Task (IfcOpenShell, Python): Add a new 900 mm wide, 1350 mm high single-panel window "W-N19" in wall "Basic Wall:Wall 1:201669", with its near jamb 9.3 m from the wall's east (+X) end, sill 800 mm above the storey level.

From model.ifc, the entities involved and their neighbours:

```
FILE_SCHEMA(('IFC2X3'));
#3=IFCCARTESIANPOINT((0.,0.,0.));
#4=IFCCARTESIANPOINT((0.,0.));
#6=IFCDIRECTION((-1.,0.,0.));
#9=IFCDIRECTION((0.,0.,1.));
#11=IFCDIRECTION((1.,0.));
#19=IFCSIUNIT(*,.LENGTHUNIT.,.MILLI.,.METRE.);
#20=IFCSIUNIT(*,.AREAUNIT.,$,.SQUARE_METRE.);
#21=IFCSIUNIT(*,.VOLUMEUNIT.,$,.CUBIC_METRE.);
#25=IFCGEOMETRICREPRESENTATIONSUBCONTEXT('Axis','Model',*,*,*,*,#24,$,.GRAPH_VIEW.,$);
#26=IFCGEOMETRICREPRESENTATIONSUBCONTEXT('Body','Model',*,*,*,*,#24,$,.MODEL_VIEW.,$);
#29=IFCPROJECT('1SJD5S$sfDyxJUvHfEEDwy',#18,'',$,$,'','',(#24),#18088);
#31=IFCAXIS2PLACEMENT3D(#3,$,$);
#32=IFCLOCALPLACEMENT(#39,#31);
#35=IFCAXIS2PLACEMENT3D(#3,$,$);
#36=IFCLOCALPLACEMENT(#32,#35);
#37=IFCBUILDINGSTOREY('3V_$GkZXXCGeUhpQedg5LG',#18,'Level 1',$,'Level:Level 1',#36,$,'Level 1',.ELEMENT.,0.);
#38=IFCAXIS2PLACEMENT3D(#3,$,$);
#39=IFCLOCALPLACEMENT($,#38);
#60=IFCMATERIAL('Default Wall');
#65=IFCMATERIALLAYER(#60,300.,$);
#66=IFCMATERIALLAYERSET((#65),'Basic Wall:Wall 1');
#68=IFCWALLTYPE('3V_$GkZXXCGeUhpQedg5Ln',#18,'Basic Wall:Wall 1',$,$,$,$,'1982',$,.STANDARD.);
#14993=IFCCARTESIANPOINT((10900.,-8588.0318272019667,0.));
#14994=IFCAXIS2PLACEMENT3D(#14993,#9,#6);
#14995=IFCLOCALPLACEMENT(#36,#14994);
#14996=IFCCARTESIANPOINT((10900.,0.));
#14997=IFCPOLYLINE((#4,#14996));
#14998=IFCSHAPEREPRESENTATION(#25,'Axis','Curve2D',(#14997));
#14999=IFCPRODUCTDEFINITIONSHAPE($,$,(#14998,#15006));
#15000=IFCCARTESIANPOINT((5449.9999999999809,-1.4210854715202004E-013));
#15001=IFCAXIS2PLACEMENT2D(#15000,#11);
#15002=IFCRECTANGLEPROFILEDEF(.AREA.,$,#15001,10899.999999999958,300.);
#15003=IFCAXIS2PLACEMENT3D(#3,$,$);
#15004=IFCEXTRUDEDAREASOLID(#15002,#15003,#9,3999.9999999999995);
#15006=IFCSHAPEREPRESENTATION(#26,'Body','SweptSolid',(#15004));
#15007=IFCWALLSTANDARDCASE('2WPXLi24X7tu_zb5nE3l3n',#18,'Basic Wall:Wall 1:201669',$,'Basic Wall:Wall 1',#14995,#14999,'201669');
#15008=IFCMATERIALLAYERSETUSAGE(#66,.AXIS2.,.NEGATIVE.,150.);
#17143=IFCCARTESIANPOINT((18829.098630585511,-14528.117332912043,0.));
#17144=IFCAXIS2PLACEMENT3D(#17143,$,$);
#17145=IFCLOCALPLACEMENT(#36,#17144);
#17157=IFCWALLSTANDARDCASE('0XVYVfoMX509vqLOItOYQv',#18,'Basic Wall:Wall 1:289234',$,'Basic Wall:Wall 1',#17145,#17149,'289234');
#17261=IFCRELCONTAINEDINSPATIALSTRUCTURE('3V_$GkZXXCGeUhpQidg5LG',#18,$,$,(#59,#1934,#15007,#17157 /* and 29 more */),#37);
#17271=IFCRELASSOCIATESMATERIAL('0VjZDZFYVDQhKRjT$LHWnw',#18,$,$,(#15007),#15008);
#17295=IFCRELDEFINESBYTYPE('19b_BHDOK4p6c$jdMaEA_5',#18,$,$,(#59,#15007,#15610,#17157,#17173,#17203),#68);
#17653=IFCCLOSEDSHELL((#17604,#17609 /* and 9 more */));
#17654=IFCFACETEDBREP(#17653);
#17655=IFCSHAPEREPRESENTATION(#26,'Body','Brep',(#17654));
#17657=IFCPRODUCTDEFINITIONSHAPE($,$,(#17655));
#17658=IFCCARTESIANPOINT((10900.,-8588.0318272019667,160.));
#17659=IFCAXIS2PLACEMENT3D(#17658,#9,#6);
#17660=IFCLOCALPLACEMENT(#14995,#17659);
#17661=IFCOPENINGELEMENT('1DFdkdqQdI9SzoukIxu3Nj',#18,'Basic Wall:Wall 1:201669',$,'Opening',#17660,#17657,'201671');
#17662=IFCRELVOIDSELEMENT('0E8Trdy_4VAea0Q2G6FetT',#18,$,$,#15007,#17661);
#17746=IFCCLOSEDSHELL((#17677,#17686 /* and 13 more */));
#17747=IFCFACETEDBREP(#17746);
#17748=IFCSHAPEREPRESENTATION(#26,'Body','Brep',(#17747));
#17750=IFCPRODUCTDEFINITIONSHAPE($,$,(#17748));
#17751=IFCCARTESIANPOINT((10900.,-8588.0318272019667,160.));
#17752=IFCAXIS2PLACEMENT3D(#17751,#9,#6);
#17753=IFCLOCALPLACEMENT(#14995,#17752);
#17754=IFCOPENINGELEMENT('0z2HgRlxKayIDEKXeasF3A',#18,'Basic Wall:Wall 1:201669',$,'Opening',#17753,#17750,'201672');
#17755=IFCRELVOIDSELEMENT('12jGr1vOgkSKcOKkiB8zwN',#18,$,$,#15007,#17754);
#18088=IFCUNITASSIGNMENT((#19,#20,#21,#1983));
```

```python
import numpy as np
import ifcopenshell
import ifcopenshell.api.feature
import ifcopenshell.api.geometry
import ifcopenshell.api.root
import ifcopenshell.api.spatial
import ifcopenshell.api.type
import ifcopenshell.geom
import ifcopenshell.util.element
import ifcopenshell.util.placement
import ifcopenshell.util.representation
import ifcopenshell.util.shape
import ifcopenshell.util.unit

model = ifcopenshell.open("model.ifc")
unit_scale = ifcopenshell.util.unit.calculate_unit_scale(model)
settings = ifcopenshell.geom.settings()


def volume(element):
    """Net volume in cubic metres, openings subtracted."""
    shape = ifcopenshell.geom.create_shape(settings, element)
    return ifcopenshell.util.shape.get_volume(shape.geometry)


wall = model.by_guid("2WPXLi24X7tu_zb5nE3l3n")
storey = ifcopenshell.util.element.get_container(wall, ifc_class="IfcBuildingStorey")
context = ifcopenshell.util.representation.get_context(model, "Model", "Body", "MODEL_VIEW")
before = volume(wall)

width, height, from_end, sill = 0.9, 1.35, 9.3, 0.8  # metres

# The wall runs along its own X axis, and the end named is its -X end.
wall_shape = ifcopenshell.geom.create_shape(settings, wall)
x, y, z = ifcopenshell.util.shape.get_vertices(wall_shape.geometry).T
start = x.min() + from_end
face, thickness = float(y.min()), float(y.max() - y.min())
wall_matrix = ifcopenshell.util.placement.get_local_placement(wall.ObjectPlacement)
level = ifcopenshell.util.placement.get_local_placement(storey.ObjectPlacement)[2, 3]


def in_wall(x, y):
    """Placement at x, y metres in the wall's axes, at sill height."""
    matrix = wall_matrix.copy()
    matrix[:, 3] = wall_matrix @ np.array([x / unit_scale, y / unit_scale, 0.0, 1.0])
    matrix[2, 3] = level + sill / unit_scale
    return matrix


# Opening: a box that overshoots both wall faces by 50 mm.
opening = ifcopenshell.api.root.create_entity(model, ifc_class="IfcOpeningElement")
box = ifcopenshell.api.geometry.add_wall_representation(
    model, context=context, length=width, height=height, thickness=thickness + 0.1
)
ifcopenshell.api.geometry.assign_representation(model, product=opening, representation=box)
ifcopenshell.api.geometry.edit_object_placement(model, product=opening, matrix=in_wall(start, face - 0.05), is_si=False)
ifcopenshell.api.feature.add_feature(model, feature=opening, element=wall)

window = ifcopenshell.api.root.create_entity(model, ifc_class="IfcWindow", name="W-N19")
window.OverallWidth, window.OverallHeight = width / unit_scale, height / unit_scale
body = ifcopenshell.api.geometry.add_window_representation(
    model,
    context=context,
    overall_width=window.OverallWidth,
    overall_height=window.OverallHeight,
    partition_type="SINGLE_PANEL",
)
ifcopenshell.api.geometry.assign_representation(model, product=window, representation=body)
ifcopenshell.api.spatial.assign_container(model, products=[window], relating_structure=storey)
fills = ifcopenshell.api.feature.add_filling(model, opening=opening, element=window)
fills.OwnerHistory = window.OwnerHistory  # required in IFC2X3

# IFC2X3 keeps the operation on the window style.
style = ifcopenshell.api.root.create_entity(model, ifc_class="IfcWindowStyle", name="W-N19")
style.OperationType, style.ConstructionType = "SINGLE_PANEL", "NOTDEFINED"
style.ParameterTakesPrecedence = style.Sizeable = False
ifcopenshell.api.type.assign_type(model, related_objects=[window], relating_type=style)

# Centre the window in the wall's thickness.
ifcopenshell.api.geometry.edit_object_placement(model, product=window, matrix=in_wall(start, face), is_si=False)
window_shape = ifcopenshell.geom.create_shape(settings, window)
depth = ifcopenshell.util.shape.get_vertices(window_shape.geometry)[:, 1]
offset = face + thickness / 2 - (depth.min() + depth.max()) / 2
ifcopenshell.api.geometry.edit_object_placement(model, product=window, matrix=in_wall(start, offset), is_si=False)

after = volume(wall)

print(f"wall volume {before:.3f} -> {after:.3f} m3")

model.write("model_rev.ifc")
```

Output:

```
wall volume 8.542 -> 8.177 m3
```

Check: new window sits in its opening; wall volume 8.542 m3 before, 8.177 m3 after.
